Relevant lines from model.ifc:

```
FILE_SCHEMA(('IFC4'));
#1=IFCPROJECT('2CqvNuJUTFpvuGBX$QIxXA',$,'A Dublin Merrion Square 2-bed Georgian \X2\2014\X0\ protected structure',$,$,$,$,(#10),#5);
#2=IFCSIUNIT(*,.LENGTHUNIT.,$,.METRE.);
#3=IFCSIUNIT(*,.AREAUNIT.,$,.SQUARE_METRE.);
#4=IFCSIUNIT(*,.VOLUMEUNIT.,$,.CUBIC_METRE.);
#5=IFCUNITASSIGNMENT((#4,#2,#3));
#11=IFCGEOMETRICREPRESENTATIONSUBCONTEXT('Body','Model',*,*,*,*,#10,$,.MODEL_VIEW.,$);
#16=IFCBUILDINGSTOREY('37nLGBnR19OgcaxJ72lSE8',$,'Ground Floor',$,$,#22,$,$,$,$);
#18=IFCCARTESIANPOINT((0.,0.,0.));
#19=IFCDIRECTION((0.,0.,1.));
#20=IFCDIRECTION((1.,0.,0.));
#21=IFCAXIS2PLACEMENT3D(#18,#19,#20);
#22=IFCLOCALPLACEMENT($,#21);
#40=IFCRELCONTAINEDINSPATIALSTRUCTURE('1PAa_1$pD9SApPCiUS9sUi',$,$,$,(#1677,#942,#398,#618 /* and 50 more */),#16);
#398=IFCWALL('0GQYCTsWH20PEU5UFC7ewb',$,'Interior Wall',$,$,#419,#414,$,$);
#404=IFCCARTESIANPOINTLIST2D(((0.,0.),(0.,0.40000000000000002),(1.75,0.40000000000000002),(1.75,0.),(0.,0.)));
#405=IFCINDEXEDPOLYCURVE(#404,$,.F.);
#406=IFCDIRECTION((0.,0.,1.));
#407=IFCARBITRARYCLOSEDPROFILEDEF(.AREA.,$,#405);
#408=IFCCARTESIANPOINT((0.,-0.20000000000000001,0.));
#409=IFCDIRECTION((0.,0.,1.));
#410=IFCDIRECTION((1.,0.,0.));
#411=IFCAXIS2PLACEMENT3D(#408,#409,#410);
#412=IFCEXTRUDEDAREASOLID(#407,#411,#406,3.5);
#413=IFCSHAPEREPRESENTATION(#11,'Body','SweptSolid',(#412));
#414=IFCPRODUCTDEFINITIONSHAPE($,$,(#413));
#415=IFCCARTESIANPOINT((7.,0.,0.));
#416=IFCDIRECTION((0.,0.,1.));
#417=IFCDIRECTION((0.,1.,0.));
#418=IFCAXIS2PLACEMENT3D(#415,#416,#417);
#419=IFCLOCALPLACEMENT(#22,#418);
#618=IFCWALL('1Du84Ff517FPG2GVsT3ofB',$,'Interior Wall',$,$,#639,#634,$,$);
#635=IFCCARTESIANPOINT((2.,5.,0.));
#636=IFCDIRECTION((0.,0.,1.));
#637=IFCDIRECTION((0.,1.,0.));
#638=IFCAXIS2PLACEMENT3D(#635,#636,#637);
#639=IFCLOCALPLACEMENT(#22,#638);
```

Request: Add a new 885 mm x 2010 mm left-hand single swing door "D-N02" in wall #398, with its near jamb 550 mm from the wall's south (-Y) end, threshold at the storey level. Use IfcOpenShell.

```python
import numpy as np
import ifcopenshell
import ifcopenshell.api.feature
import ifcopenshell.api.geometry
import ifcopenshell.api.root
import ifcopenshell.api.spatial
import ifcopenshell.geom
import ifcopenshell.util.element
import ifcopenshell.util.placement
import ifcopenshell.util.representation
import ifcopenshell.util.shape
import ifcopenshell.util.unit

model = ifcopenshell.open("model.ifc")
unit_scale = ifcopenshell.util.unit.calculate_unit_scale(model)
settings = ifcopenshell.geom.settings()


def volume(element):
    """Net volume in cubic metres, openings subtracted."""
    shape = ifcopenshell.geom.create_shape(settings, element)
    return ifcopenshell.util.shape.get_volume(shape.geometry)


wall = model.by_guid("0GQYCTsWH20PEU5UFC7ewb")
storey = ifcopenshell.util.element.get_container(wall, ifc_class="IfcBuildingStorey")
context = ifcopenshell.util.representation.get_context(model, "Model", "Body", "MODEL_VIEW")
before = volume(wall)

width, height, from_end, sill = 0.885, 2.01, 0.55, 0.0  # metres

# The wall runs along its own X axis, and the end named is its -X end.
wall_shape = ifcopenshell.geom.create_shape(settings, wall)
x, y, z = ifcopenshell.util.shape.get_vertices(wall_shape.geometry).T
start = x.min() + from_end
face, thickness = float(y.min()), float(y.max() - y.min())
wall_matrix = ifcopenshell.util.placement.get_local_placement(wall.ObjectPlacement)
level = ifcopenshell.util.placement.get_local_placement(storey.ObjectPlacement)[2, 3]


def in_wall(x, y):
    """Placement at x, y metres in the wall's axes, at sill height."""
    matrix = wall_matrix.copy()
    matrix[:, 3] = wall_matrix @ np.array([x / unit_scale, y / unit_scale, 0.0, 1.0])
    matrix[2, 3] = level + sill / unit_scale
    return matrix


# Opening: a box that overshoots both wall faces by 50 mm.
opening = ifcopenshell.api.root.create_entity(model, ifc_class="IfcOpeningElement", predefined_type="OPENING")
box = ifcopenshell.api.geometry.add_wall_representation(
    model, context=context, length=width, height=height, thickness=thickness + 0.1
)
ifcopenshell.api.geometry.assign_representation(model, product=opening, representation=box)
ifcopenshell.api.geometry.edit_object_placement(model, product=opening, matrix=in_wall(start, face - 0.05), is_si=False)
ifcopenshell.api.feature.add_feature(model, feature=opening, element=wall)

door = ifcopenshell.api.root.create_entity(model, ifc_class="IfcDoor", name="D-N02", predefined_type="DOOR")
door.OverallWidth, door.OverallHeight = width / unit_scale, height / unit_scale
door.OperationType = "SINGLE_SWING_LEFT"
body = ifcopenshell.api.geometry.add_door_representation(
    model,
    context=context,
    overall_width=door.OverallWidth,
    overall_height=door.OverallHeight,
    operation_type="SINGLE_SWING_LEFT",
    lining_properties={"LiningDepth": thickness / unit_scale, "ThresholdDepth": thickness / unit_scale},
)
ifcopenshell.api.geometry.assign_representation(model, product=door, representation=body)
ifcopenshell.api.spatial.assign_container(model, products=[door], relating_structure=storey)
ifcopenshell.api.feature.add_filling(model, opening=opening, element=door)

# The lining spans the wall, so the door starts at the wall face.
ifcopenshell.api.geometry.edit_object_placement(model, product=door, matrix=in_wall(start, face), is_si=False)

after = volume(wall)

print(f"wall volume {before:.3f} -> {after:.3f} m3")

model.write("model-out.ifc")
```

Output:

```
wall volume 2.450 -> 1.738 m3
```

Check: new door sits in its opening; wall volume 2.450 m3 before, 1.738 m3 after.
